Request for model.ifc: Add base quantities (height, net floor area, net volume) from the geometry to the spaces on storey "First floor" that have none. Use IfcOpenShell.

First a look at what the model holds.

```python
import ifcopenshell
import ifcopenshell.util.element
import ifcopenshell.util.unit

model = ifcopenshell.open("model.ifc")
print(model.schema)
for unit_type in ("LENGTHUNIT", "AREAUNIT", "VOLUMEUNIT"):
    print(unit_type, ifcopenshell.util.unit.calculate_unit_scale(model, unit_type))
storey = next(s for s in model.by_type("IfcBuildingStorey") if s.Name == "First floor")
spaces = [e for e in ifcopenshell.util.element.get_decomposition(storey) if e.is_a("IfcSpace")]
for e in sorted(spaces, key=lambda e: e.id()):
    print(e.id(), e.is_a(), e.Name, list(ifcopenshell.util.element.get_psets(e, qtos_only=True)), sep=" | ")
```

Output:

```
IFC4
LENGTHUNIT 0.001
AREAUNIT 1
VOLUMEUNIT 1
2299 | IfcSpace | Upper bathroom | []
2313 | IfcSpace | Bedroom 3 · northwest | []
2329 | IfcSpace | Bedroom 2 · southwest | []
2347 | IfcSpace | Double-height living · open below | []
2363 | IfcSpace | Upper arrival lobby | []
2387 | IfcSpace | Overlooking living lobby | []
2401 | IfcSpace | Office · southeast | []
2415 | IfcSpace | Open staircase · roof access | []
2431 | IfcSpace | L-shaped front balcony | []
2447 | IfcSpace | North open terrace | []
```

```python
import ifcopenshell
import ifcopenshell.api.pset
import ifcopenshell.geom
import ifcopenshell.util.element
import ifcopenshell.util.shape
import ifcopenshell.util.unit

model = ifcopenshell.open("model.ifc")
unit_scale = ifcopenshell.util.unit.calculate_unit_scale(model)
area_scale = ifcopenshell.util.unit.calculate_unit_scale(model, "AREAUNIT")
volume_scale = ifcopenshell.util.unit.calculate_unit_scale(model, "VOLUMEUNIT")
settings = ifcopenshell.geom.settings()

storey = next(s for s in model.by_type("IfcBuildingStorey") if s.Name == "First floor")
spaces = [e for e in ifcopenshell.util.element.get_decomposition(storey) if e.is_a("IfcSpace")]

for e in sorted(spaces, key=lambda e: e.id()):
    if ifcopenshell.util.element.get_psets(e, qtos_only=True, should_inherit=False):
        continue
    # Geometry comes back in metres, in the element's own axes.
    shape = ifcopenshell.geom.create_shape(settings, e)
    values = {
        "Height": ifcopenshell.util.shape.get_z(shape.geometry) / unit_scale,
        "NetFloorArea": ifcopenshell.util.shape.get_footprint_area(shape.geometry) / area_scale,
        "NetVolume": ifcopenshell.util.shape.get_volume(shape.geometry) / volume_scale,
    }
    qto = ifcopenshell.api.pset.add_qto(model, product=e, name="Qto_SpaceBaseQuantities")
    ifcopenshell.api.pset.edit_qto(model, qto=qto, properties=values)
    print(e.id(), {k: round(v, 3) for k, v in values.items()})

model.write("model_rev.ifc")
```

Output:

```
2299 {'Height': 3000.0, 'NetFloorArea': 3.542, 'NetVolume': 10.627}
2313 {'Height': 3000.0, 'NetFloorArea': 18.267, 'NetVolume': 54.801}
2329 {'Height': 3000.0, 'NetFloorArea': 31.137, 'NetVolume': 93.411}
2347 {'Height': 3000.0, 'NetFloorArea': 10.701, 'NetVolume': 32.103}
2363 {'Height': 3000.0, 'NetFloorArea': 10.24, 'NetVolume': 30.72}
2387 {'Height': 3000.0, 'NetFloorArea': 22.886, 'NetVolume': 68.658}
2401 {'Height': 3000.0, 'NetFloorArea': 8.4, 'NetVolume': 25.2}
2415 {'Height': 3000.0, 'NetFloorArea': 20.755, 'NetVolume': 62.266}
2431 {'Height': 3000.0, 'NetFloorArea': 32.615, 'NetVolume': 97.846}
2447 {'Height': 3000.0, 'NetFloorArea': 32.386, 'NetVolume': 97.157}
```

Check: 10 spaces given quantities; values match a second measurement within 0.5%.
